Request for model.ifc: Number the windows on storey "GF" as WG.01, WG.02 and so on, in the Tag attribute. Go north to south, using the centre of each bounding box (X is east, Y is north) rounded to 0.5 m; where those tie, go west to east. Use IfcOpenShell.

First a look at what the model holds.

```python
import ifcopenshell
import ifcopenshell.util.element
import ifcopenshell.util.placement

model = ifcopenshell.open("model.ifc")
print(model.schema)
storey = next(s for s in model.by_type("IfcBuildingStorey") if s.Name == "GF")
windows = [e for e in ifcopenshell.util.element.get_decomposition(storey) if e.is_a("IfcWindow")]
for e in sorted(windows, key=lambda e: e.id()):
    origin = ifcopenshell.util.placement.get_local_placement(e.ObjectPlacement)[:3, 3]
    print(e.id(), e.Tag, e.Name, origin.round(2) + 0.0, sep=" | ")
```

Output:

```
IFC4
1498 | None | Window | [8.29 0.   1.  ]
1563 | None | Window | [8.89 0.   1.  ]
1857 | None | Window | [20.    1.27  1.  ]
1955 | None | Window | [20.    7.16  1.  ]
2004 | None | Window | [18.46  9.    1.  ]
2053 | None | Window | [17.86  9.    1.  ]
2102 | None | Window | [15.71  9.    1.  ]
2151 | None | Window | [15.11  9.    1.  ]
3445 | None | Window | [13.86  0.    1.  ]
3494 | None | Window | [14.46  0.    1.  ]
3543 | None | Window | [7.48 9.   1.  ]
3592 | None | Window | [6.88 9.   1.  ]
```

```python
import ifcopenshell
import ifcopenshell.geom
import ifcopenshell.util.element
import ifcopenshell.util.shape

model = ifcopenshell.open("model.ifc")
settings = ifcopenshell.geom.settings()
settings.set("use-world-coords", True)


def centre(element):
    shape = ifcopenshell.geom.create_shape(settings, element)
    return ifcopenshell.util.shape.get_bbox_centroid(shape.geometry)


storey = next(s for s in model.by_type("IfcBuildingStorey") if s.Name == "GF")
windows = [e for e in ifcopenshell.util.element.get_decomposition(storey) if e.is_a("IfcWindow")]

# Insertion points can sit at a corner or the storey origin, so sort by the geometry (in metres).
centres = {e: centre(e) for e in windows}
windows.sort(key=lambda e: (-round(centres[e][1] / 0.5), centres[e][0]))

for i, e in enumerate(windows, start=1):
    number = f"WG.{i:02d}"
    e.Tag = number
    print(e.id(), number)

model.write("model_edited.ifc")
```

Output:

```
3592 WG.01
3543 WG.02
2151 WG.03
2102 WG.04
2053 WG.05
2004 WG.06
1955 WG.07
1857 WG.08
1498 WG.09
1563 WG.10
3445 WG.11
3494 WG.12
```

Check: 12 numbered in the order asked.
